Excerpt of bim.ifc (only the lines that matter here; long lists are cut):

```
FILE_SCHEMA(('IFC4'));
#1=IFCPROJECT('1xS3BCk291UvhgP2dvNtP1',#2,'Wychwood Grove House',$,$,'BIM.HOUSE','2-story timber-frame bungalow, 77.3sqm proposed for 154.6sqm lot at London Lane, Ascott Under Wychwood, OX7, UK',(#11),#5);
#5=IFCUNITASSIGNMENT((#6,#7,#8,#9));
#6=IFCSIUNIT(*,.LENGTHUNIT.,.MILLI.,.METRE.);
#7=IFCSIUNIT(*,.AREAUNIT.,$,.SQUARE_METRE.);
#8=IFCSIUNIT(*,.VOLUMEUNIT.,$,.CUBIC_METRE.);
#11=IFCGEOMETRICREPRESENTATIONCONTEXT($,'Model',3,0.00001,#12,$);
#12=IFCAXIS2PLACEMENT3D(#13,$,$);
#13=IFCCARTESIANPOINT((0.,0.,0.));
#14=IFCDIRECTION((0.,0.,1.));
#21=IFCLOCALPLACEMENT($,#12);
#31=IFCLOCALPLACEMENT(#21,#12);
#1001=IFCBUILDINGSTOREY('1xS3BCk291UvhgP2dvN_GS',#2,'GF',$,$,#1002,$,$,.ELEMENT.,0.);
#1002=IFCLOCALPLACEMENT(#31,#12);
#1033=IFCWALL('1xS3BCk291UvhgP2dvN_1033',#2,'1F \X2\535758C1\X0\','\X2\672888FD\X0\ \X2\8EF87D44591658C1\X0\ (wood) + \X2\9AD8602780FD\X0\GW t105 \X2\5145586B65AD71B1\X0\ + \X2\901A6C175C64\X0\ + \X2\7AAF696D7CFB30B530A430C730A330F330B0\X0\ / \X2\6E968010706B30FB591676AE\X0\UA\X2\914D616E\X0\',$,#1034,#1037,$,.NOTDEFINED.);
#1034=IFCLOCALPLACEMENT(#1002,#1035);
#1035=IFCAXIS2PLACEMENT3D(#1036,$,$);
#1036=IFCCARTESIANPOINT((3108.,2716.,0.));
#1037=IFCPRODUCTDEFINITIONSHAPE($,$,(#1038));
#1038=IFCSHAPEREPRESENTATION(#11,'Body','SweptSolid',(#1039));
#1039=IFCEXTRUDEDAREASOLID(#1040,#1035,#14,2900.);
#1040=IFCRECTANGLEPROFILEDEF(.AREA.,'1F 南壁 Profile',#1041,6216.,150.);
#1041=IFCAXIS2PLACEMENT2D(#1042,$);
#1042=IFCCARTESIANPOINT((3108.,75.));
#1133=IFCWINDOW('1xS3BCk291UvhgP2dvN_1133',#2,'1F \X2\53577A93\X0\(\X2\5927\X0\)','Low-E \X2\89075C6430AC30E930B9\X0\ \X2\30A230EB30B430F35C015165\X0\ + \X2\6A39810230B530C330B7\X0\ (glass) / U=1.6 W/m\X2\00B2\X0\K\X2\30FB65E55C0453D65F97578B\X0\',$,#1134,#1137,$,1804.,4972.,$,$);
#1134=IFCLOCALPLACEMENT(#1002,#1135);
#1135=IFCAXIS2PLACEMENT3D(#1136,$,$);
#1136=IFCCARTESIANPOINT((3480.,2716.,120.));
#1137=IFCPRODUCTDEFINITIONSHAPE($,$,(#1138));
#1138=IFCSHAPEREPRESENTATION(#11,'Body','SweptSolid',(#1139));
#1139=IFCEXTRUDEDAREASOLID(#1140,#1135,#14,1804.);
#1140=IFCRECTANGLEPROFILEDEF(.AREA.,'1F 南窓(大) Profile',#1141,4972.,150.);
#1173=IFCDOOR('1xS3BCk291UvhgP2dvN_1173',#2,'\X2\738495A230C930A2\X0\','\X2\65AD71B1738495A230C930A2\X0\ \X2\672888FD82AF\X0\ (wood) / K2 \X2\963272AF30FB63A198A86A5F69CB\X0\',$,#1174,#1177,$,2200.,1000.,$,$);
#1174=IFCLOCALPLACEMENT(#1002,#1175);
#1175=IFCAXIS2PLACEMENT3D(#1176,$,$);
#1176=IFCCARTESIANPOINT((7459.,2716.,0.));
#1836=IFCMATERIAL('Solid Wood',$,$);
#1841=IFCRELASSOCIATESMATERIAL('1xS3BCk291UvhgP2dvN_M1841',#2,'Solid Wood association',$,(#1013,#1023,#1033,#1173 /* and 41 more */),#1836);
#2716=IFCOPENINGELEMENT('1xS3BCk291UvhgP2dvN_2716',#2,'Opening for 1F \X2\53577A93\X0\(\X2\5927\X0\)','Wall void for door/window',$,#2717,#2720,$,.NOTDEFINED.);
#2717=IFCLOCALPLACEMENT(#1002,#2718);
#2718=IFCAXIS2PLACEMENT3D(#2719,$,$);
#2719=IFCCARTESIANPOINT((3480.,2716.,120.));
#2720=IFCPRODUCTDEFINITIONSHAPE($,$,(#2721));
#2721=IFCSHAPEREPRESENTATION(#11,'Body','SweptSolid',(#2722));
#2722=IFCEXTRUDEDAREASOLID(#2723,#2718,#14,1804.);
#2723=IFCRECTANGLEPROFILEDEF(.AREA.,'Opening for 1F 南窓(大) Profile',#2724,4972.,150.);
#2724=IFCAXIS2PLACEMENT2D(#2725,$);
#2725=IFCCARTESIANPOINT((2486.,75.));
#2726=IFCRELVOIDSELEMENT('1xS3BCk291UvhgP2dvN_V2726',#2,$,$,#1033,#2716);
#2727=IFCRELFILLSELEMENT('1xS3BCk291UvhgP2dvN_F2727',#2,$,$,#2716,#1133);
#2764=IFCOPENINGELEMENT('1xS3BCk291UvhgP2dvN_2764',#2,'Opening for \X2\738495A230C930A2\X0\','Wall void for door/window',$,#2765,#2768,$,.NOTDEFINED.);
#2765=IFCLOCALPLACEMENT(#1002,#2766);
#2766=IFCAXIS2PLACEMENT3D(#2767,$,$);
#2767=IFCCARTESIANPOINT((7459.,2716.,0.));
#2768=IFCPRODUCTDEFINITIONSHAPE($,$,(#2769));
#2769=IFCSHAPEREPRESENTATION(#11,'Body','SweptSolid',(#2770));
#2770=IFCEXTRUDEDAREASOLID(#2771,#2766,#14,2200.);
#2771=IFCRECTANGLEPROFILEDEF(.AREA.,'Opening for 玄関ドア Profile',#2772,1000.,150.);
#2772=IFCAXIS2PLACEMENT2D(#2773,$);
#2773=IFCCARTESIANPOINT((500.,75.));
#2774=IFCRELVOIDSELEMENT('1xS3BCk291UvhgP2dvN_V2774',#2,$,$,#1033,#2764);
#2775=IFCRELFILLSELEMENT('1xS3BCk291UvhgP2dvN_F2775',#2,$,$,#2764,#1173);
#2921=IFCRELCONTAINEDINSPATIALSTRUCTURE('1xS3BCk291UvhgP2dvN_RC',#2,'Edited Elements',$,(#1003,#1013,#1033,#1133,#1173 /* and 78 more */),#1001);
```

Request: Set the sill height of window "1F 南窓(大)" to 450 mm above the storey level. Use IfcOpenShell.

```python
import numpy as np
import ifcopenshell
import ifcopenshell.api.geometry
import ifcopenshell.geom
import ifcopenshell.util.element
import ifcopenshell.util.placement
import ifcopenshell.util.shape
import ifcopenshell.util.unit

model = ifcopenshell.open("bim.ifc")
unit_scale = ifcopenshell.util.unit.calculate_unit_scale(model)

window = model.by_id(1133)
opening = window.FillsVoids[0].RelatingOpeningElement
storey = ifcopenshell.util.element.get_container(window, ifc_class="IfcBuildingStorey")
level = ifcopenshell.util.placement.get_local_placement(storey.ObjectPlacement)[2, 3]

# The opening's origin need not be at the sill, so measure its lowest point.
shape = ifcopenshell.geom.create_shape(ifcopenshell.geom.settings(), opening)
bottom = ifcopenshell.util.shape.get_shape_bottom_elevation(shape, shape.geometry) / unit_scale
dz = level + 450.0 - bottom

shift = np.array([0.0, 0.0, dz])
# The window is not placed relative to its opening, so move both.
for product in (opening, window):
    matrix = ifcopenshell.util.placement.get_local_placement(product.ObjectPlacement)
    matrix[:3, 3] += shift
    ifcopenshell.api.geometry.edit_object_placement(model, product=product, matrix=matrix, is_si=False)

print(f"moved by {dz * unit_scale:+.3f} m")

model.write("bim-out.ifc")
```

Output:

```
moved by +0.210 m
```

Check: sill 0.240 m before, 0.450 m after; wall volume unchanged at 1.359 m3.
